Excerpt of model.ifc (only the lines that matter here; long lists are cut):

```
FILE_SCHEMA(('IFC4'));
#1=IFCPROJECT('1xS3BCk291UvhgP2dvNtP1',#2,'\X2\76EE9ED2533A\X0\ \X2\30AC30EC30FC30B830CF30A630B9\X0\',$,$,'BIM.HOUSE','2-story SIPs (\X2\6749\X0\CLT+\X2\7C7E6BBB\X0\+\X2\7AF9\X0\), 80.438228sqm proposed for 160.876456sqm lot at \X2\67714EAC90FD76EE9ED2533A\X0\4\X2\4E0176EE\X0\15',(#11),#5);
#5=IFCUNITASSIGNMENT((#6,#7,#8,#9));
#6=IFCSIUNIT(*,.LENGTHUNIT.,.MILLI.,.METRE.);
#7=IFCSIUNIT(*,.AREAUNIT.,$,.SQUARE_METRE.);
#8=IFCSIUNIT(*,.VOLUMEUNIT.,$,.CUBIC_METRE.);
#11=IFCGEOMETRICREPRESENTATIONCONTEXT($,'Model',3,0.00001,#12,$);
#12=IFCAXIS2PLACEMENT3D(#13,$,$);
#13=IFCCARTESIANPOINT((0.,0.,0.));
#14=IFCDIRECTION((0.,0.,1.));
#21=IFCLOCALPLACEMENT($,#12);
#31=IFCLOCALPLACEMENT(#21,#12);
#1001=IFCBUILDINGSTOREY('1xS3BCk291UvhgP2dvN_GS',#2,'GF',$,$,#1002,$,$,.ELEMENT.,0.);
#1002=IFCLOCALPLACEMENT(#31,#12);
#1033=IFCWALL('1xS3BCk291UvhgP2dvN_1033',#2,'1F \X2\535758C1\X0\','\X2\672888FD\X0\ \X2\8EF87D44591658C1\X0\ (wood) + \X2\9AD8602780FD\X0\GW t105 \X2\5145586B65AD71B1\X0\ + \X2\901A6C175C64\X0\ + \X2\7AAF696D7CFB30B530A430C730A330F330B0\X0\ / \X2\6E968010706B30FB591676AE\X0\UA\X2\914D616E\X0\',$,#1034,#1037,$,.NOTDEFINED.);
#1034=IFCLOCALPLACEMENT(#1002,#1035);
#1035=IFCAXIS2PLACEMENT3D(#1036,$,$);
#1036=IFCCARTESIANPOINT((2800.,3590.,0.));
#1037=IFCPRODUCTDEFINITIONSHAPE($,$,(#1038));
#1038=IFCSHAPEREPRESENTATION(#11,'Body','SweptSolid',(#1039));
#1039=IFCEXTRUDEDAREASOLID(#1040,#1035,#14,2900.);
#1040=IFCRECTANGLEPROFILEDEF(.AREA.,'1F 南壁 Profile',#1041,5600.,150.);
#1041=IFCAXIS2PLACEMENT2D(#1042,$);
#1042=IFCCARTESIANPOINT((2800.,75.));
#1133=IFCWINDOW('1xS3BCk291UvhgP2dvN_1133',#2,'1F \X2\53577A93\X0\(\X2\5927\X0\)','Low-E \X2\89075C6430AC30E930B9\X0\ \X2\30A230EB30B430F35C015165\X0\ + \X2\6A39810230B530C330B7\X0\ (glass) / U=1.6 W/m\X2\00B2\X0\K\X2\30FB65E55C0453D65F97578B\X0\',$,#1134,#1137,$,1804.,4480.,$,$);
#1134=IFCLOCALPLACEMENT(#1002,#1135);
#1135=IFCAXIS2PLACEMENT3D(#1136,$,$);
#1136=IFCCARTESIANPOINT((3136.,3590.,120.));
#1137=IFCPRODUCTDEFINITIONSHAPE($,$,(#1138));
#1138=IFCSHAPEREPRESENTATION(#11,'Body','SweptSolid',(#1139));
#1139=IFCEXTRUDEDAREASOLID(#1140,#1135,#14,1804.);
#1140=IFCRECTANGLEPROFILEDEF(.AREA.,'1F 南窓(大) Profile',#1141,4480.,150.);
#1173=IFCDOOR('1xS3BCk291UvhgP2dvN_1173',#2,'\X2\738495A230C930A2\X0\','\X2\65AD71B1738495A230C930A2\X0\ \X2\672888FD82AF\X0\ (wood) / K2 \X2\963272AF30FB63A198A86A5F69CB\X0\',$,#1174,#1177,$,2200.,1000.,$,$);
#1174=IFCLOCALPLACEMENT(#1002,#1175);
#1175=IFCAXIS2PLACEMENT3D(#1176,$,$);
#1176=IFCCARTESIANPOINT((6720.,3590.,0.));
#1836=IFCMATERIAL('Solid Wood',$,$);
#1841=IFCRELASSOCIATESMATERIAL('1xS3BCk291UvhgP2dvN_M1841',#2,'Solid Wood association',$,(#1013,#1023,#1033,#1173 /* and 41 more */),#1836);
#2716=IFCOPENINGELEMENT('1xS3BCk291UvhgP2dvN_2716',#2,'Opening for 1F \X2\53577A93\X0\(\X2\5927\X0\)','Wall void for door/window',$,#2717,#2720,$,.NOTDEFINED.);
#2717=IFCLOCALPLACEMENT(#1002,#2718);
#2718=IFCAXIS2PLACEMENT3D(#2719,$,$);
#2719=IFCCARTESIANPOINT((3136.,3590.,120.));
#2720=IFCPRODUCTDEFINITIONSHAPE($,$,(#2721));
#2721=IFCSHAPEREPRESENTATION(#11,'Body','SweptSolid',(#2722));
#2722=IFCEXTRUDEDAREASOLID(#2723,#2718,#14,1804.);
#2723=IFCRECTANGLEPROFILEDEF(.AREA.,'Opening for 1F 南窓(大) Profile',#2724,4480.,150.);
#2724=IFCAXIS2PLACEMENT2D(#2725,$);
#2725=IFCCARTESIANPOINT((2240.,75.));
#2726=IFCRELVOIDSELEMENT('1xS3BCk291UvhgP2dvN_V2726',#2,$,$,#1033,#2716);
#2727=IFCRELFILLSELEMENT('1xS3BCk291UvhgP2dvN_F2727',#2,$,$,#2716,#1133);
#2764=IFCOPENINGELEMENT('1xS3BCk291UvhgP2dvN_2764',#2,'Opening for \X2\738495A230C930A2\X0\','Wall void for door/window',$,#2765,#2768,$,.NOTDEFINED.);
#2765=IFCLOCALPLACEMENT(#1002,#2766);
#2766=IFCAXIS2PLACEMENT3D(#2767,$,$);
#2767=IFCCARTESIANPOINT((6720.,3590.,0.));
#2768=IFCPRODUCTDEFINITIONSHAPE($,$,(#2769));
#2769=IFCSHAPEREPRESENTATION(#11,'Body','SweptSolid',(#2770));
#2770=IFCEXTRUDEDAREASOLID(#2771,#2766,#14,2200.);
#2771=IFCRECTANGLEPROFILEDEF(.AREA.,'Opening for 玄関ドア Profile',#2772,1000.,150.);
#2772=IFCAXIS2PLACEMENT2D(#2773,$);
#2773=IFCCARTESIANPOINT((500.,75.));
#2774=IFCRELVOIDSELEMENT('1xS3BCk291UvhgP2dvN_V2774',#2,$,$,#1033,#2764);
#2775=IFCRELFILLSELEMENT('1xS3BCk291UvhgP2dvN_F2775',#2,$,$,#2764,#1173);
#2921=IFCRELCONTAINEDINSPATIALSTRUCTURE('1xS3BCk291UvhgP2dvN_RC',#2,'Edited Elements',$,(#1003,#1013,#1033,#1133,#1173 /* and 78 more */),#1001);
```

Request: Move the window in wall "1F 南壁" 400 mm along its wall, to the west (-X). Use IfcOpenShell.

```python
import ifcopenshell
import ifcopenshell.api.geometry
import ifcopenshell.util.placement

model = ifcopenshell.open("model.ifc")

window = model.by_guid("1xS3BCk291UvhgP2dvN_1133")
opening = window.FillsVoids[0].RelatingOpeningElement
wall = opening.VoidsElements[0].RelatingBuildingElement

wall_matrix = ifcopenshell.util.placement.get_local_placement(wall.ObjectPlacement)
shift = wall_matrix[:3, 0] * -400.0
before = ifcopenshell.util.placement.get_local_placement(window.ObjectPlacement)[:3, 3].copy()

# The window is not placed relative to its opening, so move both.
for product in (opening, window):
    matrix = ifcopenshell.util.placement.get_local_placement(product.ObjectPlacement)
    matrix[:3, 3] += shift
    ifcopenshell.api.geometry.edit_object_placement(model, product=product, matrix=matrix, is_si=False)

after = ifcopenshell.util.placement.get_local_placement(window.ObjectPlacement)[:3, 3]
print("window moved by", (after - before).round(3) + 0.0)

model.write("model-out.ifc")
```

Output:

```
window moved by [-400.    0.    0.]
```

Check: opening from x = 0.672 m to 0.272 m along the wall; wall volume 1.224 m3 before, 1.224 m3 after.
